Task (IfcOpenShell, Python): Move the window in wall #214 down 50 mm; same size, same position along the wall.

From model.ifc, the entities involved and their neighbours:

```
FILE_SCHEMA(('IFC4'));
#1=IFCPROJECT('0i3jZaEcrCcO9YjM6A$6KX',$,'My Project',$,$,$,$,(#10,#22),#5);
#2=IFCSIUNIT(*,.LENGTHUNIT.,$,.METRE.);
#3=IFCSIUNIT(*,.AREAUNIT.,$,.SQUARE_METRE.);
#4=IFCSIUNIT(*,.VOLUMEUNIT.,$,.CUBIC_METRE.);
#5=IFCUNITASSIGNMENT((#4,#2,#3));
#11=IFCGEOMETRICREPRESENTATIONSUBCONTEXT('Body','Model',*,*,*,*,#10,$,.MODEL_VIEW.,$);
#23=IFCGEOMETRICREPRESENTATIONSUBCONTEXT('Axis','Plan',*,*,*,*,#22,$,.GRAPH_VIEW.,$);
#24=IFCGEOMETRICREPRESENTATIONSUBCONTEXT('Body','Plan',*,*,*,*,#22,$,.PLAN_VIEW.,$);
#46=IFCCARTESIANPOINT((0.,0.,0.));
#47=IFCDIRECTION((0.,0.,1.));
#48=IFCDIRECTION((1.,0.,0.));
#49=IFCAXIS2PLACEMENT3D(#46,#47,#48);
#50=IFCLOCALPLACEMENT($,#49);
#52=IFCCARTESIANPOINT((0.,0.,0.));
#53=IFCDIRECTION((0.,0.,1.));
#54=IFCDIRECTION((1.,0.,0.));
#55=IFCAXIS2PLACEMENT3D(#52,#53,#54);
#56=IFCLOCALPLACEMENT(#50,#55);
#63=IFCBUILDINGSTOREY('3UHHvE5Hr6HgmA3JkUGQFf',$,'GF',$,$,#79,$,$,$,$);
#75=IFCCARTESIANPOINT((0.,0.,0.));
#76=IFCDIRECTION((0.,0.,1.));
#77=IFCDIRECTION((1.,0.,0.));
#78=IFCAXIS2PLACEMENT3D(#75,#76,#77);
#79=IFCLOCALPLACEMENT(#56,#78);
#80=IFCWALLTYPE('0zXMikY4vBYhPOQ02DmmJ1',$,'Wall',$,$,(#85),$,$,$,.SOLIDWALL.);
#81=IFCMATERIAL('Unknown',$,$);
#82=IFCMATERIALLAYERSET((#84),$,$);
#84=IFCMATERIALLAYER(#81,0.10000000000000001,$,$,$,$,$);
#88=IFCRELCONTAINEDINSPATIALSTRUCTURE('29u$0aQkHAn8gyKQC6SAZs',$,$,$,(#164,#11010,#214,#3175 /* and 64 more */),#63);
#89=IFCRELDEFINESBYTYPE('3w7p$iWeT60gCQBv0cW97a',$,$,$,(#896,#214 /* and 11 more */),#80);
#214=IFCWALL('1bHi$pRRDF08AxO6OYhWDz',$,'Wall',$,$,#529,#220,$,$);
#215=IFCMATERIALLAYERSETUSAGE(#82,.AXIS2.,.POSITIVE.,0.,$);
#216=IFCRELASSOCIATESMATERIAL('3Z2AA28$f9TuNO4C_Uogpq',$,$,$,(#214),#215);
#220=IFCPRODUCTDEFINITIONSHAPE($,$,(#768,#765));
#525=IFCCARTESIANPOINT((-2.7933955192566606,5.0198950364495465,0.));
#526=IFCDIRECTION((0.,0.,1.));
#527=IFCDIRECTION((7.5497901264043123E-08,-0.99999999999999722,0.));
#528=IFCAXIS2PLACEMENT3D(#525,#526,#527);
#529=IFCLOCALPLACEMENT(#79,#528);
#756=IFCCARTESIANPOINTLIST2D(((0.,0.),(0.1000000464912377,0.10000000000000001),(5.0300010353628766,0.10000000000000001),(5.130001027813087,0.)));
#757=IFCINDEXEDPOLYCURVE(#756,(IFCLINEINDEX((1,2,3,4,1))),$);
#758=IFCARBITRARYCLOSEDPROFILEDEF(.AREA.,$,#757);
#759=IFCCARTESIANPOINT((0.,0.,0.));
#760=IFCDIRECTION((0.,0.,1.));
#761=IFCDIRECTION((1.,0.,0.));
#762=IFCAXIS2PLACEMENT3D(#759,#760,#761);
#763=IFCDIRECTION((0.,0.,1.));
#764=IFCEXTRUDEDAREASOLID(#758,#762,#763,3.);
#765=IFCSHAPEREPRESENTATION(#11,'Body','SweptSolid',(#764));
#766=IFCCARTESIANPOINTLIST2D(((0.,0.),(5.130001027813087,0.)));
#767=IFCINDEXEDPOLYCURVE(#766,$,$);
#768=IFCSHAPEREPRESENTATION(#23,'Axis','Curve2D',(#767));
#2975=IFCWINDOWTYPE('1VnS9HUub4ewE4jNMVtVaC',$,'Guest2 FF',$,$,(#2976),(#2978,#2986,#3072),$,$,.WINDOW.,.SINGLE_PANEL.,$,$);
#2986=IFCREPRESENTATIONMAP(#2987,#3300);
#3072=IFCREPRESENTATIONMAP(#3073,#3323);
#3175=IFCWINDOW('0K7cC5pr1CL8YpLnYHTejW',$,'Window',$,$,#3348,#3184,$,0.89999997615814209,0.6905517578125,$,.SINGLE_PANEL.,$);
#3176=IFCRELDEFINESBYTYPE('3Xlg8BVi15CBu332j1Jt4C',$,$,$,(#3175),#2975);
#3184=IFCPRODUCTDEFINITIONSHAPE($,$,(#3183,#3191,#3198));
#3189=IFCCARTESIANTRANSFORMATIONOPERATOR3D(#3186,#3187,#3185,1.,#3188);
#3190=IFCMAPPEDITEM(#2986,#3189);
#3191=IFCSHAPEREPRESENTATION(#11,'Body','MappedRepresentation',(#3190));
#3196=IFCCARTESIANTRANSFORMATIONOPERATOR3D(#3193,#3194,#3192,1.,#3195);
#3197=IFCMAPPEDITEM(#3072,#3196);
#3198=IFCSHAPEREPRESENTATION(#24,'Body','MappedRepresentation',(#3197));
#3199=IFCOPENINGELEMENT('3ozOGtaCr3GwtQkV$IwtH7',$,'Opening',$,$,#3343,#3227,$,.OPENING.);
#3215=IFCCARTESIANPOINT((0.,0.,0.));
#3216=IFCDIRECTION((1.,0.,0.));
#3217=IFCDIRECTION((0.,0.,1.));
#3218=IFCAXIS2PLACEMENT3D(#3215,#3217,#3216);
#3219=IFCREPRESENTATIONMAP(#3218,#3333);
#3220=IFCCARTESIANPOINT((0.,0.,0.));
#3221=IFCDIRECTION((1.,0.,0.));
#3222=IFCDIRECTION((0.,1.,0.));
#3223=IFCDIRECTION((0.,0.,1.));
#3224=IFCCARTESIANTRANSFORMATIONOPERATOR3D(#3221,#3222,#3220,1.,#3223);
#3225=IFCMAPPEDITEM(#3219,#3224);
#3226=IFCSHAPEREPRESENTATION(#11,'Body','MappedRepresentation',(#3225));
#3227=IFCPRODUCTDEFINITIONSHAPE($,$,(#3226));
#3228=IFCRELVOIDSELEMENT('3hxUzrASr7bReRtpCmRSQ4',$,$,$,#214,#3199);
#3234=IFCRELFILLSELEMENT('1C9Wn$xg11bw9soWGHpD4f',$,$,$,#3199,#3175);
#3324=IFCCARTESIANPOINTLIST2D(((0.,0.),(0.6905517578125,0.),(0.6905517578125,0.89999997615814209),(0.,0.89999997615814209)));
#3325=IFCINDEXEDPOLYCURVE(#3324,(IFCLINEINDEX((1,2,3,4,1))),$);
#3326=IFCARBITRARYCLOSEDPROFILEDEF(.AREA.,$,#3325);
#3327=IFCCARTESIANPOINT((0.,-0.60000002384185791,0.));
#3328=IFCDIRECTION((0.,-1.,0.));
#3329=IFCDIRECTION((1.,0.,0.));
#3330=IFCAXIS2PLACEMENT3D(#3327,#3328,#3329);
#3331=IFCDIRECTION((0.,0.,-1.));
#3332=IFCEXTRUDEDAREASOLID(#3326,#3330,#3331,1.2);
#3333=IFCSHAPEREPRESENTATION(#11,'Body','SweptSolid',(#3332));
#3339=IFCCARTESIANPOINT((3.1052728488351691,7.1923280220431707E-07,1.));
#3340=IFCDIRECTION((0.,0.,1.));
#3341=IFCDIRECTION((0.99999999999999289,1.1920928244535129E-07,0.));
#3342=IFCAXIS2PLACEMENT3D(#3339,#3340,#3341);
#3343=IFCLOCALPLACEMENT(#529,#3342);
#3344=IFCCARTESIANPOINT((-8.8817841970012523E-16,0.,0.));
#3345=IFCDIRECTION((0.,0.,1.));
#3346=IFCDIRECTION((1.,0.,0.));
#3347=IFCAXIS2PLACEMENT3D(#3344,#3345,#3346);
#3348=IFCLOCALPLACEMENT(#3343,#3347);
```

```python
import numpy as np
import ifcopenshell
import ifcopenshell.api.geometry
import ifcopenshell.util.placement
import ifcopenshell.util.unit

model = ifcopenshell.open("model.ifc")
unit_scale = ifcopenshell.util.unit.calculate_unit_scale(model)

window = model.by_guid("0K7cC5pr1CL8YpLnYHTejW")
opening = window.FillsVoids[0].RelatingOpeningElement
dz = -0.05 / unit_scale

shift = np.array([0.0, 0.0, dz])
# The window is placed relative to its opening, so it follows when the opening moves.
matrix = ifcopenshell.util.placement.get_local_placement(opening.ObjectPlacement)
matrix[:3, 3] += shift
ifcopenshell.api.geometry.edit_object_placement(
    model, product=opening, matrix=matrix, is_si=False, should_transform_children=True
)

print(f"moved by {dz * unit_scale:+.3f} m")

model.write("model_rev.ifc")
```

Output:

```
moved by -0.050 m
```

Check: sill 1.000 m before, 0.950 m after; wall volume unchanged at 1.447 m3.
